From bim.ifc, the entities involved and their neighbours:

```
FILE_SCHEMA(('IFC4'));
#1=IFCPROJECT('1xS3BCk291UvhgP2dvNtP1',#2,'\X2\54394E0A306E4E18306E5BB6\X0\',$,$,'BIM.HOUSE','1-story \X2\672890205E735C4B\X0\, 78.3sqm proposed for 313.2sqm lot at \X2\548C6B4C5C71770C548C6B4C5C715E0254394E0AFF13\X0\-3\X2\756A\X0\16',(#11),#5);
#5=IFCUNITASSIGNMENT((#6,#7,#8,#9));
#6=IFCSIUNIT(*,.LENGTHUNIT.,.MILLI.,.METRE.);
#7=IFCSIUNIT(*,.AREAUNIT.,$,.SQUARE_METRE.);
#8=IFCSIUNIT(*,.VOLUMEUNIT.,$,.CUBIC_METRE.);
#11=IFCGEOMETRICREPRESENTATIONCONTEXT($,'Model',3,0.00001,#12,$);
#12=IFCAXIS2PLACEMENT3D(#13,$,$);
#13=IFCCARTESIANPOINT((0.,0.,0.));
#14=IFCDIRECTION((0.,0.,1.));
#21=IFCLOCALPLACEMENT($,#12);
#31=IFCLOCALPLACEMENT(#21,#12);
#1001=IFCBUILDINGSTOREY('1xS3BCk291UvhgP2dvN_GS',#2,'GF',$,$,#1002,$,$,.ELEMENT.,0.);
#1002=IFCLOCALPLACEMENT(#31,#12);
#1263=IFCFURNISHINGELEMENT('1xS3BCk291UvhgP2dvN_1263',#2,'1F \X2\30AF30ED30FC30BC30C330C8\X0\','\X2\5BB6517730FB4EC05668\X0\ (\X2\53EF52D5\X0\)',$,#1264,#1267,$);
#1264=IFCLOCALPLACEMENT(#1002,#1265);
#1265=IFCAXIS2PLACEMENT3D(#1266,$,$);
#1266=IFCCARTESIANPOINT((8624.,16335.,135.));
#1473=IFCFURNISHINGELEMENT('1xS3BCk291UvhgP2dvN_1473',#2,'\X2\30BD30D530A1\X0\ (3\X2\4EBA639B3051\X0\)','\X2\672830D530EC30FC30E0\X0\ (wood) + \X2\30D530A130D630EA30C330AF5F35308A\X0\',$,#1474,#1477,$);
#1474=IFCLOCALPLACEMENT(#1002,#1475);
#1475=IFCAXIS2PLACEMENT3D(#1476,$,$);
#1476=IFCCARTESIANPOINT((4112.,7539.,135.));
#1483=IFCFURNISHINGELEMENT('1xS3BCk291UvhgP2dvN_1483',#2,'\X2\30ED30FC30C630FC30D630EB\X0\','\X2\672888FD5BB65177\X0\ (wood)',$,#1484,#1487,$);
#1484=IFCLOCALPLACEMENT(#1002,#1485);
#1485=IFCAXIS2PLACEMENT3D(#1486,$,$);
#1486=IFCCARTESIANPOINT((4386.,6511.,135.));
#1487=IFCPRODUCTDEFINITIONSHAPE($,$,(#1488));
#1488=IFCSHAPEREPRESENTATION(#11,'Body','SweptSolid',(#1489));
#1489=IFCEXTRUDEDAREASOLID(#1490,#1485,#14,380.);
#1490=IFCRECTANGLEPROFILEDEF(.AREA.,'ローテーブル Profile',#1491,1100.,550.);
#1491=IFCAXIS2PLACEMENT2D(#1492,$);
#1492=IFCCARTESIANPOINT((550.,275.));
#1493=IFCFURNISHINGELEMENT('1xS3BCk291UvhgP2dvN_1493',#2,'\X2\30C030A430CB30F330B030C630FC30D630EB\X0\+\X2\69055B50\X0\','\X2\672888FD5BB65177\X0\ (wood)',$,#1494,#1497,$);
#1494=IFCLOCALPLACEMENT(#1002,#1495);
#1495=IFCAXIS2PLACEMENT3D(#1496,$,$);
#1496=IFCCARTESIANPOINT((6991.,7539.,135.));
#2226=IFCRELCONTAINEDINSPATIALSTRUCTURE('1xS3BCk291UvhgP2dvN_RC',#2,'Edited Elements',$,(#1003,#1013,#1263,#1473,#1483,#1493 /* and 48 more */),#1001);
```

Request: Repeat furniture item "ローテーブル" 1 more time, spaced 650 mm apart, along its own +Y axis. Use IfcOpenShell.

```python
import ifcopenshell
import ifcopenshell.api.geometry
import ifcopenshell.api.root
import ifcopenshell.util.element
import ifcopenshell.util.placement
import ifcopenshell.util.unit

model = ifcopenshell.open("bim.ifc")
unit_scale = ifcopenshell.util.unit.calculate_unit_scale(model)


def reuse_history(source, copy):
    """copy_class also copies each property set's owner history, people and application; keep the originals."""
    for rel in copy.IsDefinedBy:
        if rel.is_a("IfcRelDefinesByProperties") and (history := rel.RelatingPropertyDefinition.OwnerHistory):
            rel.RelatingPropertyDefinition.OwnerHistory = source.OwnerHistory
            ifcopenshell.util.element.remove_deep2(model, history)


source = model.by_id(1483)
base = ifcopenshell.util.placement.get_local_placement(source.ObjectPlacement)
step = base[:3, 1] * 0.65 / unit_scale

for i in range(1, 2):
    copy = ifcopenshell.api.root.copy_class(model, product=source)
    copy.Representation = ifcopenshell.util.element.copy_deep(
        model, source.Representation, exclude=["IfcGeometricRepresentationContext", "IfcRepresentationMap"]
    )
    reuse_history(source, copy)
    matrix = base.copy()
    matrix[:3, 3] += i * step
    print("added at", matrix[:3, 3].round(3) + 0.0)
    ifcopenshell.api.geometry.edit_object_placement(model, product=copy, matrix=matrix, is_si=False)

model.write("bim_rev.ifc")
```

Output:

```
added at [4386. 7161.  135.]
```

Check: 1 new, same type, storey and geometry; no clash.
